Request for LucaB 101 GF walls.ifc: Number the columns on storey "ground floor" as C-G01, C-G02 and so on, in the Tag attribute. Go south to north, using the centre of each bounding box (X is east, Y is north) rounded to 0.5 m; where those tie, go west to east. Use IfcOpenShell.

First a look at what the model holds.

```python
import ifcopenshell
import ifcopenshell.util.element
import ifcopenshell.util.placement

model = ifcopenshell.open("LucaB 101 GF walls.ifc")
print(model.schema)
storey = next(s for s in model.by_type("IfcBuildingStorey") if s.Name == "ground floor")
columns = [e for e in ifcopenshell.util.element.get_decomposition(storey) if e.is_a("IfcColumn")]
for e in sorted(columns, key=lambda e: e.id()):
    origin = ifcopenshell.util.placement.get_local_placement(e.ObjectPlacement)[:3, 3]
    print(e.id(), e.Tag, e.Name, origin.round(2) + 0.0, sep=" | ")
```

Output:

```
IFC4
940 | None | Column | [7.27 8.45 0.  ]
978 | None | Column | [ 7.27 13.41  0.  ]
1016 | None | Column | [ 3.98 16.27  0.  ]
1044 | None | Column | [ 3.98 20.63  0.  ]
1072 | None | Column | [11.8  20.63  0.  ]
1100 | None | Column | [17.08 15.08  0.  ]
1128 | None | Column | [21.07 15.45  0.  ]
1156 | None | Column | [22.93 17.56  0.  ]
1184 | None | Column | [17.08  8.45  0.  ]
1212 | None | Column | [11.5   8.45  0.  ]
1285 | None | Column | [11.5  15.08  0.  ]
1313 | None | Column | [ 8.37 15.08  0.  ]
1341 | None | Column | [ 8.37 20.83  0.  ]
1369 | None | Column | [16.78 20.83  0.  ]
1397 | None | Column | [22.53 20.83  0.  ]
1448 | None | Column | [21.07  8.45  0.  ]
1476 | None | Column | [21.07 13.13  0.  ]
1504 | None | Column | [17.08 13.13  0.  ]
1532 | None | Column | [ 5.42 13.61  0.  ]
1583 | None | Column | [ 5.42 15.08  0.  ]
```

```python
import ifcopenshell
import ifcopenshell.geom
import ifcopenshell.util.element
import ifcopenshell.util.shape

model = ifcopenshell.open("LucaB 101 GF walls.ifc")
settings = ifcopenshell.geom.settings()
settings.set("use-world-coords", True)


def centre(element):
    shape = ifcopenshell.geom.create_shape(settings, element)
    return ifcopenshell.util.shape.get_bbox_centroid(shape.geometry)


storey = next(s for s in model.by_type("IfcBuildingStorey") if s.Name == "ground floor")
columns = [e for e in ifcopenshell.util.element.get_decomposition(storey) if e.is_a("IfcColumn")]

# Insertion points can sit at a corner or the storey origin, so sort by the geometry (in metres).
centres = {e: centre(e) for e in columns}
columns.sort(key=lambda e: (round(centres[e][1] / 0.5), centres[e][0]))

for i, e in enumerate(columns, start=1):
    number = f"C-G{i:02d}"
    e.Tag = number
    print(e.id(), number)

model.write("LucaB 101 GF walls_updated.ifc")
```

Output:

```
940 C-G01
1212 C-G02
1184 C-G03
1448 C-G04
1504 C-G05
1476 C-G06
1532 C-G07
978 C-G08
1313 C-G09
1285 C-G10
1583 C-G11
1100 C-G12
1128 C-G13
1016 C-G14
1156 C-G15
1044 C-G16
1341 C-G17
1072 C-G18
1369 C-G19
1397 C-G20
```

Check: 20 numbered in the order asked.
